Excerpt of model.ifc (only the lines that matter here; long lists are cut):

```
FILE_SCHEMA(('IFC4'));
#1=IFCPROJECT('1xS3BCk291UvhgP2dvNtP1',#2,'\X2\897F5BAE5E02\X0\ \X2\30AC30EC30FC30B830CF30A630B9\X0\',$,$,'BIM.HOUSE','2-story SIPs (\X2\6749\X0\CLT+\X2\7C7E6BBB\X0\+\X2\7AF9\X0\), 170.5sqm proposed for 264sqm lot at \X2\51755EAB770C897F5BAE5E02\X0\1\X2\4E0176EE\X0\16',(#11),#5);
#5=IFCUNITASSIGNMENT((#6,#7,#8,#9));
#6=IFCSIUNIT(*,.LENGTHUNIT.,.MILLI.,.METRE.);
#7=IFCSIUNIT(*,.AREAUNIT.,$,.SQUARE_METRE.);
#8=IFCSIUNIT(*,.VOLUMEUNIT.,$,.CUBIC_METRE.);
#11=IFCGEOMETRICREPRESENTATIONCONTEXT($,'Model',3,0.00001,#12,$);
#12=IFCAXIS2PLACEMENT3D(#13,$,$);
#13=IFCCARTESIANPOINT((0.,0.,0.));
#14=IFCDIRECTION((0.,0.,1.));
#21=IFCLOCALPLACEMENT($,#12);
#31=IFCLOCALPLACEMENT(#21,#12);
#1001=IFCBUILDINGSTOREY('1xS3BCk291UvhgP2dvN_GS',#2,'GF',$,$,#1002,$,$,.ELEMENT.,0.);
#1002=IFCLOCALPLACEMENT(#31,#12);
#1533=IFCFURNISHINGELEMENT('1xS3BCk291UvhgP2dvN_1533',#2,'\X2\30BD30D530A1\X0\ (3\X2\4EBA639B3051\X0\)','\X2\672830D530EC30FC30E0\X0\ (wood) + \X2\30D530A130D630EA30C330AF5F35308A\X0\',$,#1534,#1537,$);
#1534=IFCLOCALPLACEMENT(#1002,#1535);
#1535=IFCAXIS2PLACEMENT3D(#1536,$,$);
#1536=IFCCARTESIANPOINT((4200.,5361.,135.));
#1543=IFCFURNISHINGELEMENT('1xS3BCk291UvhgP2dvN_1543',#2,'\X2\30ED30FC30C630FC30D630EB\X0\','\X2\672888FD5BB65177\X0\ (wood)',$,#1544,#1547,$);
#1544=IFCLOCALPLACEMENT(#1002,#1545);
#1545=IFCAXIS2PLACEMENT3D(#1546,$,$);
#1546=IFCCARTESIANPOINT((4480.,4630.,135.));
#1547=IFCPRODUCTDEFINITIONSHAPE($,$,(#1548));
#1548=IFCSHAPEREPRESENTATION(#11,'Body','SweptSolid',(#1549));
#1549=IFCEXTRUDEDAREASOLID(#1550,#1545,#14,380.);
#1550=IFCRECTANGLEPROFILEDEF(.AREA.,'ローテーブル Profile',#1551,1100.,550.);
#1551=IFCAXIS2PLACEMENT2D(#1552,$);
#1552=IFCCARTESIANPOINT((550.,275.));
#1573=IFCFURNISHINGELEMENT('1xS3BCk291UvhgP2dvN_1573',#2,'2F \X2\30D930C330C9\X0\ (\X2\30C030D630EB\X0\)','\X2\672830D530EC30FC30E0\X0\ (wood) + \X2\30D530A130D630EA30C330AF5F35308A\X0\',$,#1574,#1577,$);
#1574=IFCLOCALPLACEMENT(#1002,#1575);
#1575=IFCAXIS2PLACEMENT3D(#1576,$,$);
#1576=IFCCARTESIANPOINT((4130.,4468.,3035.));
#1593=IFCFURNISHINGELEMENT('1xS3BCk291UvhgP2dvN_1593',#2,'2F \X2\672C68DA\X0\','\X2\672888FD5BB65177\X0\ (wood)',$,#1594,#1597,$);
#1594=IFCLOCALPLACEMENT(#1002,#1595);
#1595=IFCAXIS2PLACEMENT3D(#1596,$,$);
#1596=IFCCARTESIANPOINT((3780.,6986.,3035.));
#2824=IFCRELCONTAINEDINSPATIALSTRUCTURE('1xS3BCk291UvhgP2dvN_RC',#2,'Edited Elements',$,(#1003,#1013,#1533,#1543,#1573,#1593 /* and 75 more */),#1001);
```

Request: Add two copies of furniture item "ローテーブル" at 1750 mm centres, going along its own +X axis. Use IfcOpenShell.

```python
import ifcopenshell
import ifcopenshell.api.geometry
import ifcopenshell.api.root
import ifcopenshell.util.element
import ifcopenshell.util.placement

model = ifcopenshell.open("model.ifc")


def reuse_history(source, copy):
    """copy_class also copies each property set's owner history, people and application; keep the originals."""
    for rel in copy.IsDefinedBy:
        if rel.is_a("IfcRelDefinesByProperties") and (history := rel.RelatingPropertyDefinition.OwnerHistory):
            rel.RelatingPropertyDefinition.OwnerHistory = source.OwnerHistory
            ifcopenshell.util.element.remove_deep2(model, history)


source = model.by_guid("1xS3BCk291UvhgP2dvN_1543")
base = ifcopenshell.util.placement.get_local_placement(source.ObjectPlacement)
step = base[:3, 0] * 1750.0

for i in range(1, 3):
    copy = ifcopenshell.api.root.copy_class(model, product=source)
    copy.Representation = ifcopenshell.util.element.copy_deep(
        model, source.Representation, exclude=["IfcGeometricRepresentationContext", "IfcRepresentationMap"]
    )
    reuse_history(source, copy)
    matrix = base.copy()
    matrix[:3, 3] += i * step
    print("added at", matrix[:3, 3].round(3) + 0.0)
    ifcopenshell.api.geometry.edit_object_placement(model, product=copy, matrix=matrix, is_si=False)

model.write("model_updated.ifc")
```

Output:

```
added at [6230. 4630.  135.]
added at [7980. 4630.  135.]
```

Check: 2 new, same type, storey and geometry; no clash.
